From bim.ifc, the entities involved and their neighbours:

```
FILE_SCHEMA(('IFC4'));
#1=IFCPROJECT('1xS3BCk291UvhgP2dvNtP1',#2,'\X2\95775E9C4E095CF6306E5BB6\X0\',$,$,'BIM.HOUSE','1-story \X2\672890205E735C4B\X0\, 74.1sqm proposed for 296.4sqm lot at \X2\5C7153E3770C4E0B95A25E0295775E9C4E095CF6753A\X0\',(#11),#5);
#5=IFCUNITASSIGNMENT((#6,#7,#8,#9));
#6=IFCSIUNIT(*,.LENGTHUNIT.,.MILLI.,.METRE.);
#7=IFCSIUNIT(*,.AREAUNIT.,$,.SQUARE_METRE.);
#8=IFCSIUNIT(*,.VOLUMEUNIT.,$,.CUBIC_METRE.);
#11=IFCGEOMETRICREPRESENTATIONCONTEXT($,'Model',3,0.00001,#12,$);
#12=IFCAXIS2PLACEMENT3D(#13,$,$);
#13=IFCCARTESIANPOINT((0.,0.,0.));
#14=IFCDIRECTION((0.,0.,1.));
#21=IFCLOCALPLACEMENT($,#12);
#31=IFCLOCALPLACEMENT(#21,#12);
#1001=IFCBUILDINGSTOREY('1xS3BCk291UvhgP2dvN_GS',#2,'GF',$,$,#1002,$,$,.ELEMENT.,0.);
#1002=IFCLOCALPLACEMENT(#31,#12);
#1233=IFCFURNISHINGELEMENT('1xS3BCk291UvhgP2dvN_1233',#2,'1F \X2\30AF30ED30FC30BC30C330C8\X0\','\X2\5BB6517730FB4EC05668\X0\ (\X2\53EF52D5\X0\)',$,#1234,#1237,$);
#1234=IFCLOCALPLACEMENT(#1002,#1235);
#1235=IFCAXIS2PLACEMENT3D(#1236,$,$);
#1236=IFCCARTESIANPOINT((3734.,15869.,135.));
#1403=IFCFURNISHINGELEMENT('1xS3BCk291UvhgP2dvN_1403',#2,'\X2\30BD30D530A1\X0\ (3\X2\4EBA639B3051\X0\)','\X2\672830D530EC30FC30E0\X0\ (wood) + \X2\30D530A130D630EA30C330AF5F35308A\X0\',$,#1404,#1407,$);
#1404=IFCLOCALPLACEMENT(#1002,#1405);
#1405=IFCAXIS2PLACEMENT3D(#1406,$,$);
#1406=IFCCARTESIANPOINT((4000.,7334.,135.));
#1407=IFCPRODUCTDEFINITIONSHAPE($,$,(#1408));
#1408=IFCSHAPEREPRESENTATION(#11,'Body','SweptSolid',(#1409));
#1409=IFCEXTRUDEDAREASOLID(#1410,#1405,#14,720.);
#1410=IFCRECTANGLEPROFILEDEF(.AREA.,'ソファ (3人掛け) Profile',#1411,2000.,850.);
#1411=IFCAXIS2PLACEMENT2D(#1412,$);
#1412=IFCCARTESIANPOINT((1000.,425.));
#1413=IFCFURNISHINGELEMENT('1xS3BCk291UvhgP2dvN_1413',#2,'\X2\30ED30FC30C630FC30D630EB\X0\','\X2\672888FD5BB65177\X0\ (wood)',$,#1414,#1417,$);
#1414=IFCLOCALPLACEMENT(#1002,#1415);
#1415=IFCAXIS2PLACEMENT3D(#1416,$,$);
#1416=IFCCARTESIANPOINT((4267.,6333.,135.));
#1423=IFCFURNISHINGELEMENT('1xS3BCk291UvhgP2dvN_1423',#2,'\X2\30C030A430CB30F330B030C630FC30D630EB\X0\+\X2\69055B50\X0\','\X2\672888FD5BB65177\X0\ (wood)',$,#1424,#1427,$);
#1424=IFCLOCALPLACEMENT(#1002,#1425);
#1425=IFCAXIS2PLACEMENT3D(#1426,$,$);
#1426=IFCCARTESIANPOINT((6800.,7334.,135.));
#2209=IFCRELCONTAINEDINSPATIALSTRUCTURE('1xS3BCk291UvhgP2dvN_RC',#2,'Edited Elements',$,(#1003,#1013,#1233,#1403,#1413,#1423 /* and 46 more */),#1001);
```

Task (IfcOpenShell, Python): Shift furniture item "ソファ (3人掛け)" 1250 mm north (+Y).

```python
import ifcopenshell
import ifcopenshell.api.geometry
import ifcopenshell.util.placement

model = ifcopenshell.open("bim.ifc")

item = model.by_id(1403)
matrix = ifcopenshell.util.placement.get_local_placement(item.ObjectPlacement)
matrix[1, 3] += 1250.0
ifcopenshell.api.geometry.edit_object_placement(model, product=item, matrix=matrix, is_si=False)

print(ifcopenshell.util.placement.get_local_placement(item.ObjectPlacement).round(3) + 0.0)

model.write("bim_rev.ifc")
```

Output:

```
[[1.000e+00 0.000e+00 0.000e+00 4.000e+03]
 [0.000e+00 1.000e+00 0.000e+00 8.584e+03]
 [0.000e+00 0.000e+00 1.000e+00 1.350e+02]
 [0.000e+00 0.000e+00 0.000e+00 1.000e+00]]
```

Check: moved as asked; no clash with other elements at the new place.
